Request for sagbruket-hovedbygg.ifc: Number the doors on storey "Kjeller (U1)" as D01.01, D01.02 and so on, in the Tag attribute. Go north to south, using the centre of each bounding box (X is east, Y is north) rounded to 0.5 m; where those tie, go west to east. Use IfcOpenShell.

First a look at what the model holds.

```python
import ifcopenshell
import ifcopenshell.util.element
import ifcopenshell.util.placement

model = ifcopenshell.open("sagbruket-hovedbygg.ifc")
print(model.schema)
storey = next(s for s in model.by_type("IfcBuildingStorey") if s.Name == "Kjeller (U1)")
doors = [e for e in ifcopenshell.util.element.get_decomposition(storey) if e.is_a("IfcDoor")]
for e in sorted(doors, key=lambda e: e.id()):
    origin = ifcopenshell.util.placement.get_local_placement(e.ObjectPlacement)[:3, 3]
    print(e.id(), e.Tag, e.Name, origin.round(2) + 0.0, sep=" | ")
```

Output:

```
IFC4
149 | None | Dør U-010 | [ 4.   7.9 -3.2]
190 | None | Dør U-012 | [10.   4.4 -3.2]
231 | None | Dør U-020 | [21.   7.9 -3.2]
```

```python
import ifcopenshell
import ifcopenshell.geom
import ifcopenshell.util.element
import ifcopenshell.util.shape

model = ifcopenshell.open("sagbruket-hovedbygg.ifc")
settings = ifcopenshell.geom.settings()
settings.set("use-world-coords", True)


def centre(element):
    shape = ifcopenshell.geom.create_shape(settings, element)
    return ifcopenshell.util.shape.get_bbox_centroid(shape.geometry)


storey = next(s for s in model.by_type("IfcBuildingStorey") if s.Name == "Kjeller (U1)")
doors = [e for e in ifcopenshell.util.element.get_decomposition(storey) if e.is_a("IfcDoor")]

# Insertion points can sit at a corner or the storey origin, so sort by the geometry (in metres).
centres = {e: centre(e) for e in doors}
doors.sort(key=lambda e: (-round(centres[e][1] / 0.5), centres[e][0]))

for i, e in enumerate(doors, start=1):
    number = f"D01.{i:02d}"
    e.Tag = number
    print(e.id(), number)

model.write("sagbruket-hovedbygg-out.ifc")
```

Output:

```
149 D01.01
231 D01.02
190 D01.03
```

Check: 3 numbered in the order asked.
